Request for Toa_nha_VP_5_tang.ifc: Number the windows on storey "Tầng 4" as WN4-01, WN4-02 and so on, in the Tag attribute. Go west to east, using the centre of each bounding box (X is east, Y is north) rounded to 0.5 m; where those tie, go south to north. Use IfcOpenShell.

First a look at what the model holds.

```python
import ifcopenshell
import ifcopenshell.util.element
import ifcopenshell.util.placement

model = ifcopenshell.open("Toa_nha_VP_5_tang.ifc")
print(model.schema)
storey = next(s for s in model.by_type("IfcBuildingStorey") if s.Name == "Tầng 4")
windows = [e for e in ifcopenshell.util.element.get_decomposition(storey) if e.is_a("IfcWindow")]
for e in sorted(windows, key=lambda e: e.id()):
    origin = ifcopenshell.util.placement.get_local_placement(e.ObjectPlacement)[:3, 3]
    print(e.id(), e.Tag, e.Name, origin.round(2) + 0.0, sep=" | ")
```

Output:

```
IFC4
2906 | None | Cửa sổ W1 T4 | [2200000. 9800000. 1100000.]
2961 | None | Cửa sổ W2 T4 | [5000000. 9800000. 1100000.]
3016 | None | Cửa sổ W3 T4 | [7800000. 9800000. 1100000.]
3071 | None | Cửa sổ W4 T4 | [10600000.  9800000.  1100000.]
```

```python
import ifcopenshell
import ifcopenshell.geom
import ifcopenshell.util.element
import ifcopenshell.util.shape

model = ifcopenshell.open("Toa_nha_VP_5_tang.ifc")
settings = ifcopenshell.geom.settings()
settings.set("use-world-coords", True)


def centre(element):
    shape = ifcopenshell.geom.create_shape(settings, element)
    return ifcopenshell.util.shape.get_bbox_centroid(shape.geometry)


storey = next(s for s in model.by_type("IfcBuildingStorey") if s.Name == "Tầng 4")
windows = [e for e in ifcopenshell.util.element.get_decomposition(storey) if e.is_a("IfcWindow")]

# Insertion points can sit at a corner or the storey origin, so sort by the geometry (in metres).
centres = {e: centre(e) for e in windows}
windows.sort(key=lambda e: (round(centres[e][0] / 0.5), centres[e][1]))

for i, e in enumerate(windows, start=1):
    number = f"WN4-{i:02d}"
    e.Tag = number
    print(e.id(), number)

model.write("Toa_nha_VP_5_tang_rev.ifc")
```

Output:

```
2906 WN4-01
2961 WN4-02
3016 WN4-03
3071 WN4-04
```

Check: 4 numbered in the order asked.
